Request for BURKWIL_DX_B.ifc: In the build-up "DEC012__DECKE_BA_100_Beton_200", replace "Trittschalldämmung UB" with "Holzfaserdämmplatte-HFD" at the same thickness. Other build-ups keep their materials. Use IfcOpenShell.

First a look at what the model holds.

```python
import ifcopenshell
import ifcopenshell.util.element

model = ifcopenshell.open("BURKWIL_DX_B.ifc")
print(model.schema)
for layer_set in model.by_type("IfcMaterialLayerSet"):
    if layer_set.LayerSetName == "DEC012__DECKE_BA_100_Beton_200":
        for layer in layer_set.MaterialLayers:
            print(layer.id(), layer.Material and layer.Material.Name, layer.LayerThickness, sep=" | ")
        print(len(ifcopenshell.util.element.get_elements_by_material(model, layer_set)), "elements and types use it")
print(sorted(m.Name for m in model.by_type("IfcMaterial") if m.Name)[:60])
```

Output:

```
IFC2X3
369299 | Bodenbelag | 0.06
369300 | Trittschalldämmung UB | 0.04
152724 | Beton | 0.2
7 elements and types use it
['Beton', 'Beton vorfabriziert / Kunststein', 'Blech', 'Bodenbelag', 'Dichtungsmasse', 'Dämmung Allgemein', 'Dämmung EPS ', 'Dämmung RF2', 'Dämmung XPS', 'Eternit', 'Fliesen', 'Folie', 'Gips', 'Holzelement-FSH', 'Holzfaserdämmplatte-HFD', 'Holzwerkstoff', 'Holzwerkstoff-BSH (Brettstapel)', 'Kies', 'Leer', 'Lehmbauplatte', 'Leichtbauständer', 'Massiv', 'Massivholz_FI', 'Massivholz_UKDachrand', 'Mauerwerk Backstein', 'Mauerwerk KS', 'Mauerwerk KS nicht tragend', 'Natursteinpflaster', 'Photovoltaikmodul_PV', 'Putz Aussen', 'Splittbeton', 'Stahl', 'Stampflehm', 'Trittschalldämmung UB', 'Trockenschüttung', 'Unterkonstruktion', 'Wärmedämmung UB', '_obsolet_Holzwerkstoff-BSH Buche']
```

```python
import ifcopenshell
import ifcopenshell.api.material

model = ifcopenshell.open("BURKWIL_DX_B.ifc")

layer_set = next(s for s in model.by_type("IfcMaterialLayerSet") if s.LayerSetName == "DEC012__DECKE_BA_100_Beton_200")
layer = next(l for l in layer_set.MaterialLayers if l.Material and l.Material.Name == "Trittschalldämmung UB")
material = next(m for m in model.by_type("IfcMaterial") if m.Name == "Holzfaserdämmplatte-HFD")

# Point this one layer at the other material; renaming the old one would change it everywhere.
ifcopenshell.api.material.edit_layer(model, layer=layer, attributes={}, material=material)

print([l.Material.Name if l.Material else None for l in layer_set.MaterialLayers])

model.write("BURKWIL_DX_B_edited.ifc")
```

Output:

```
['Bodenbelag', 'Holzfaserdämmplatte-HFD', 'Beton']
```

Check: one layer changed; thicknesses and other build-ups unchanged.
